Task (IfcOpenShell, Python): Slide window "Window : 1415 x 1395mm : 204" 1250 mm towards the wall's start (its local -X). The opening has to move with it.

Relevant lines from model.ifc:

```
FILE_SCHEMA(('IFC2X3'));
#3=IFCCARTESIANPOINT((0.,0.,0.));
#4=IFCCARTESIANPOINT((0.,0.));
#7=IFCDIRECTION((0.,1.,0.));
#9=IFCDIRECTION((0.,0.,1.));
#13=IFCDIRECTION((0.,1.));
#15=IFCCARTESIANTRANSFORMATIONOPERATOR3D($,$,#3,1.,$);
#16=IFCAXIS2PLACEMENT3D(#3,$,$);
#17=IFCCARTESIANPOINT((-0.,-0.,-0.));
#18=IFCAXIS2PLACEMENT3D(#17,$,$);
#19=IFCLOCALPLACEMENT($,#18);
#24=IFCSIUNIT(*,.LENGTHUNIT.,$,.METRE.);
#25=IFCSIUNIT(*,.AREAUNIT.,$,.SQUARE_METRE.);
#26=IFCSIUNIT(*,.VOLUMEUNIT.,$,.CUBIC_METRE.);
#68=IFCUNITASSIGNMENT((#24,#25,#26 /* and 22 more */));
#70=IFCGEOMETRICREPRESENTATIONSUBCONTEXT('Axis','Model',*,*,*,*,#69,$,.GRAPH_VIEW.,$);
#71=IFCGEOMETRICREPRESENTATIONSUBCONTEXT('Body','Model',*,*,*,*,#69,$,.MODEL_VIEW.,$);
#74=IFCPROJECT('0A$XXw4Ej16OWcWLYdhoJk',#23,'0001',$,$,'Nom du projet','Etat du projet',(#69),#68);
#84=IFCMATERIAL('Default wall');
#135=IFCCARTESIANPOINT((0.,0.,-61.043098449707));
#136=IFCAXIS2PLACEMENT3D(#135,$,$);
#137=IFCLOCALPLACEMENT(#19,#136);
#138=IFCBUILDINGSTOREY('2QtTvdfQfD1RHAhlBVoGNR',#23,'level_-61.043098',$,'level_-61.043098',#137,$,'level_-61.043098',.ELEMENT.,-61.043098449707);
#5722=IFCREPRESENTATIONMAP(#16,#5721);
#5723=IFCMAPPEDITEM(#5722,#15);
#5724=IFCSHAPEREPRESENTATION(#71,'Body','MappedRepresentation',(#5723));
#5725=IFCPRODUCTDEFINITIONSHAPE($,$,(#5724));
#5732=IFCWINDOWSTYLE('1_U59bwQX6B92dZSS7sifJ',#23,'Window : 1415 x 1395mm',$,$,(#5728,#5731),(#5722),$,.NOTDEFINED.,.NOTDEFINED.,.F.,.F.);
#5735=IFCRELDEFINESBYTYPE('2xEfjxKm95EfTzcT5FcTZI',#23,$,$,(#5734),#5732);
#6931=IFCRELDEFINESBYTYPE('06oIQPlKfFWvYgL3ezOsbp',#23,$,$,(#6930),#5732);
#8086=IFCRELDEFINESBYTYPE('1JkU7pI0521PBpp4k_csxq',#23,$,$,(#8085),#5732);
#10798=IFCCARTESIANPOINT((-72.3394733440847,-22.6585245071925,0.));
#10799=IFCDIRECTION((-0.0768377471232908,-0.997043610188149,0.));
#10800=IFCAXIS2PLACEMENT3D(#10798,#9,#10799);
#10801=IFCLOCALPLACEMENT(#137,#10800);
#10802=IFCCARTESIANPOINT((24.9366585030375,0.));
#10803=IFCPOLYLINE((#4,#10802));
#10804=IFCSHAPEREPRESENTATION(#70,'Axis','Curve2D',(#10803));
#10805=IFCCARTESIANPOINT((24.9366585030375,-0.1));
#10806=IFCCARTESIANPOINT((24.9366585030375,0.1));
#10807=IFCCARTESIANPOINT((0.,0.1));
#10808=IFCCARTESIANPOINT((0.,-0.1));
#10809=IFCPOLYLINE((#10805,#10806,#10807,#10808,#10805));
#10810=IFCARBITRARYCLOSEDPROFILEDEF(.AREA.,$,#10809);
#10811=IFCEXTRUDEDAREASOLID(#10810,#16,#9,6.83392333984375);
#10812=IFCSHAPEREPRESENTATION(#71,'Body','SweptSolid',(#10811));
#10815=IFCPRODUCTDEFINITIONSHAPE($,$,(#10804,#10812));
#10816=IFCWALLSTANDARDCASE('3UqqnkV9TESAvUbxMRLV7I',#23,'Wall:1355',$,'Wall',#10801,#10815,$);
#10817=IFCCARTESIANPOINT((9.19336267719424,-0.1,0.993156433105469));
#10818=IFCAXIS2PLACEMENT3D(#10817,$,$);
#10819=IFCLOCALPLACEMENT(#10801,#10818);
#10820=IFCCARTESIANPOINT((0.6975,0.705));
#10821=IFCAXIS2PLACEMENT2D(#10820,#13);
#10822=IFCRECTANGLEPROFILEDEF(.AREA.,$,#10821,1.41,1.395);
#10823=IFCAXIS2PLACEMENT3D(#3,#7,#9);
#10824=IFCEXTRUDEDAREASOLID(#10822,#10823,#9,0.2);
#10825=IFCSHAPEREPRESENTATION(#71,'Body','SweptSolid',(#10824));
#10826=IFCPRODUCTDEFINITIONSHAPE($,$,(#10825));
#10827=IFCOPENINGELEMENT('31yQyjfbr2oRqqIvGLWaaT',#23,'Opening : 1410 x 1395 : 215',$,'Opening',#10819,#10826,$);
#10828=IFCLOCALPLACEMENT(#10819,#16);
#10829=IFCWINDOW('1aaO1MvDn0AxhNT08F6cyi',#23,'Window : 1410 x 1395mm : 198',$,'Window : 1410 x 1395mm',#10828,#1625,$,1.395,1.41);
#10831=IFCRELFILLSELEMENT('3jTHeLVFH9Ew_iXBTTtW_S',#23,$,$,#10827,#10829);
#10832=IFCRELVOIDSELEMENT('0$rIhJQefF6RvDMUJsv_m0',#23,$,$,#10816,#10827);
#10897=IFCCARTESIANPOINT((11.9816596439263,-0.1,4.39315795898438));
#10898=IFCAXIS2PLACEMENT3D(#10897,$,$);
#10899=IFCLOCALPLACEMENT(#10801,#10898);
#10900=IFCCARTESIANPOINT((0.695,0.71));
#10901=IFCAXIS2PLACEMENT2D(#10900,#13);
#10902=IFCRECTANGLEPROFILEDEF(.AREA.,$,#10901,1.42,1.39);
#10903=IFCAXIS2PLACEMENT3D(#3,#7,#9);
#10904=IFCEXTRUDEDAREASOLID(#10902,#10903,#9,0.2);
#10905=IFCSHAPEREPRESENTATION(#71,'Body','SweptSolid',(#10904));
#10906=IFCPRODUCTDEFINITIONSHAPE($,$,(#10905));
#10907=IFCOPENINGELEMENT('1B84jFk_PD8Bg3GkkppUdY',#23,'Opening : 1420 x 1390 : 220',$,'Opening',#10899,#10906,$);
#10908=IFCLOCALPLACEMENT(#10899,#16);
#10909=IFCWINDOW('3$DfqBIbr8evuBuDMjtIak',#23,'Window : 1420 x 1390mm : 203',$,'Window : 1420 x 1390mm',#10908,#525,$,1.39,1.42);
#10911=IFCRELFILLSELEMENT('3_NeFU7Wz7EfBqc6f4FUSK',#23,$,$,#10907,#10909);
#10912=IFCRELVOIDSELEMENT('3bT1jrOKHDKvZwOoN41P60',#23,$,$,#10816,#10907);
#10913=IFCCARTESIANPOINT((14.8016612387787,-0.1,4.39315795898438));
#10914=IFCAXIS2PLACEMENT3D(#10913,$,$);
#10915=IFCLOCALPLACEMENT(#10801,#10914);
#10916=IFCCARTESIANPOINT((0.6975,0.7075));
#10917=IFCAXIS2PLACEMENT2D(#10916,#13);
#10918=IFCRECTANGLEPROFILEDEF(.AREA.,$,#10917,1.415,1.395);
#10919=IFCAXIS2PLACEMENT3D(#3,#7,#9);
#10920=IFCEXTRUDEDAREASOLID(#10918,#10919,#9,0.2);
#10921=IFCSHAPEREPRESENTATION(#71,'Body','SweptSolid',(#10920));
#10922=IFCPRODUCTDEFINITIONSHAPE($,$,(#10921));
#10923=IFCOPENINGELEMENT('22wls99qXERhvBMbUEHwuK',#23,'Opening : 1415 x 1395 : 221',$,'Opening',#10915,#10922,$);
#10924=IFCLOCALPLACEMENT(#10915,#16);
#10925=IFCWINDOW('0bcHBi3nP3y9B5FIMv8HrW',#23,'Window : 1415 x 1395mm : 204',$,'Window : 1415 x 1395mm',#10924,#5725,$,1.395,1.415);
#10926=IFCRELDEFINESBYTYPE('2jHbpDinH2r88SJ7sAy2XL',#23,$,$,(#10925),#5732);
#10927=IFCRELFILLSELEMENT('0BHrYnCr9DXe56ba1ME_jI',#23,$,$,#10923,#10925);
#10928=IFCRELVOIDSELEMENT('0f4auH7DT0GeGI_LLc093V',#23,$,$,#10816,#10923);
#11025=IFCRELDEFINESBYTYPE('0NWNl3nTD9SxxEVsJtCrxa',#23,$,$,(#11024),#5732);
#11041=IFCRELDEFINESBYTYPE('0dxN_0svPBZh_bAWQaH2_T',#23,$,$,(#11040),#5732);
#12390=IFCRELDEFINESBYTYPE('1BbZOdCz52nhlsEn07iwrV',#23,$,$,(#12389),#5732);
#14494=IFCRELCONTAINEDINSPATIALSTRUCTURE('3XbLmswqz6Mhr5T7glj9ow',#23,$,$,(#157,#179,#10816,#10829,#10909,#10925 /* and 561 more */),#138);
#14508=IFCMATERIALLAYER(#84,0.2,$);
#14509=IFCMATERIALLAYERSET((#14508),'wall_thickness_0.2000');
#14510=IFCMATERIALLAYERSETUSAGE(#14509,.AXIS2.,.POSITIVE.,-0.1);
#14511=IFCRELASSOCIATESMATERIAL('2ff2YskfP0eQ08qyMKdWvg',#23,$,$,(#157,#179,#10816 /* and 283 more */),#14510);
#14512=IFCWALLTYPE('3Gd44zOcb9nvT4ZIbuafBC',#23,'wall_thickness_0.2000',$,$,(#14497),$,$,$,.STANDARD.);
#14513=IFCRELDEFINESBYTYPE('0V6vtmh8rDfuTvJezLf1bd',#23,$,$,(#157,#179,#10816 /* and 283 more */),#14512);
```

```python
import ifcopenshell
import ifcopenshell.api.geometry
import ifcopenshell.util.placement
import ifcopenshell.util.unit

model = ifcopenshell.open("model.ifc")
unit_scale = ifcopenshell.util.unit.calculate_unit_scale(model)

window = model.by_guid("0bcHBi3nP3y9B5FIMv8HrW")
opening = window.FillsVoids[0].RelatingOpeningElement
wall = opening.VoidsElements[0].RelatingBuildingElement

wall_matrix = ifcopenshell.util.placement.get_local_placement(wall.ObjectPlacement)
shift = wall_matrix[:3, 0] * -1.25 / unit_scale
before = ifcopenshell.util.placement.get_local_placement(window.ObjectPlacement)[:3, 3].copy()

# The window is placed relative to its opening, so it follows when the opening moves.
matrix = ifcopenshell.util.placement.get_local_placement(opening.ObjectPlacement)
matrix[:3, 3] += shift
ifcopenshell.api.geometry.edit_object_placement(
    model, product=opening, matrix=matrix, is_si=False, should_transform_children=True
)

after = ifcopenshell.util.placement.get_local_placement(window.ObjectPlacement)[:3, 3]
print("window moved by", (after - before).round(3) + 0.0)

model.write("model_updated.ifc")
```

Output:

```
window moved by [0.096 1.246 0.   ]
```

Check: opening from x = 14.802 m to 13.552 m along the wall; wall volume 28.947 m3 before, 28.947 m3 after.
